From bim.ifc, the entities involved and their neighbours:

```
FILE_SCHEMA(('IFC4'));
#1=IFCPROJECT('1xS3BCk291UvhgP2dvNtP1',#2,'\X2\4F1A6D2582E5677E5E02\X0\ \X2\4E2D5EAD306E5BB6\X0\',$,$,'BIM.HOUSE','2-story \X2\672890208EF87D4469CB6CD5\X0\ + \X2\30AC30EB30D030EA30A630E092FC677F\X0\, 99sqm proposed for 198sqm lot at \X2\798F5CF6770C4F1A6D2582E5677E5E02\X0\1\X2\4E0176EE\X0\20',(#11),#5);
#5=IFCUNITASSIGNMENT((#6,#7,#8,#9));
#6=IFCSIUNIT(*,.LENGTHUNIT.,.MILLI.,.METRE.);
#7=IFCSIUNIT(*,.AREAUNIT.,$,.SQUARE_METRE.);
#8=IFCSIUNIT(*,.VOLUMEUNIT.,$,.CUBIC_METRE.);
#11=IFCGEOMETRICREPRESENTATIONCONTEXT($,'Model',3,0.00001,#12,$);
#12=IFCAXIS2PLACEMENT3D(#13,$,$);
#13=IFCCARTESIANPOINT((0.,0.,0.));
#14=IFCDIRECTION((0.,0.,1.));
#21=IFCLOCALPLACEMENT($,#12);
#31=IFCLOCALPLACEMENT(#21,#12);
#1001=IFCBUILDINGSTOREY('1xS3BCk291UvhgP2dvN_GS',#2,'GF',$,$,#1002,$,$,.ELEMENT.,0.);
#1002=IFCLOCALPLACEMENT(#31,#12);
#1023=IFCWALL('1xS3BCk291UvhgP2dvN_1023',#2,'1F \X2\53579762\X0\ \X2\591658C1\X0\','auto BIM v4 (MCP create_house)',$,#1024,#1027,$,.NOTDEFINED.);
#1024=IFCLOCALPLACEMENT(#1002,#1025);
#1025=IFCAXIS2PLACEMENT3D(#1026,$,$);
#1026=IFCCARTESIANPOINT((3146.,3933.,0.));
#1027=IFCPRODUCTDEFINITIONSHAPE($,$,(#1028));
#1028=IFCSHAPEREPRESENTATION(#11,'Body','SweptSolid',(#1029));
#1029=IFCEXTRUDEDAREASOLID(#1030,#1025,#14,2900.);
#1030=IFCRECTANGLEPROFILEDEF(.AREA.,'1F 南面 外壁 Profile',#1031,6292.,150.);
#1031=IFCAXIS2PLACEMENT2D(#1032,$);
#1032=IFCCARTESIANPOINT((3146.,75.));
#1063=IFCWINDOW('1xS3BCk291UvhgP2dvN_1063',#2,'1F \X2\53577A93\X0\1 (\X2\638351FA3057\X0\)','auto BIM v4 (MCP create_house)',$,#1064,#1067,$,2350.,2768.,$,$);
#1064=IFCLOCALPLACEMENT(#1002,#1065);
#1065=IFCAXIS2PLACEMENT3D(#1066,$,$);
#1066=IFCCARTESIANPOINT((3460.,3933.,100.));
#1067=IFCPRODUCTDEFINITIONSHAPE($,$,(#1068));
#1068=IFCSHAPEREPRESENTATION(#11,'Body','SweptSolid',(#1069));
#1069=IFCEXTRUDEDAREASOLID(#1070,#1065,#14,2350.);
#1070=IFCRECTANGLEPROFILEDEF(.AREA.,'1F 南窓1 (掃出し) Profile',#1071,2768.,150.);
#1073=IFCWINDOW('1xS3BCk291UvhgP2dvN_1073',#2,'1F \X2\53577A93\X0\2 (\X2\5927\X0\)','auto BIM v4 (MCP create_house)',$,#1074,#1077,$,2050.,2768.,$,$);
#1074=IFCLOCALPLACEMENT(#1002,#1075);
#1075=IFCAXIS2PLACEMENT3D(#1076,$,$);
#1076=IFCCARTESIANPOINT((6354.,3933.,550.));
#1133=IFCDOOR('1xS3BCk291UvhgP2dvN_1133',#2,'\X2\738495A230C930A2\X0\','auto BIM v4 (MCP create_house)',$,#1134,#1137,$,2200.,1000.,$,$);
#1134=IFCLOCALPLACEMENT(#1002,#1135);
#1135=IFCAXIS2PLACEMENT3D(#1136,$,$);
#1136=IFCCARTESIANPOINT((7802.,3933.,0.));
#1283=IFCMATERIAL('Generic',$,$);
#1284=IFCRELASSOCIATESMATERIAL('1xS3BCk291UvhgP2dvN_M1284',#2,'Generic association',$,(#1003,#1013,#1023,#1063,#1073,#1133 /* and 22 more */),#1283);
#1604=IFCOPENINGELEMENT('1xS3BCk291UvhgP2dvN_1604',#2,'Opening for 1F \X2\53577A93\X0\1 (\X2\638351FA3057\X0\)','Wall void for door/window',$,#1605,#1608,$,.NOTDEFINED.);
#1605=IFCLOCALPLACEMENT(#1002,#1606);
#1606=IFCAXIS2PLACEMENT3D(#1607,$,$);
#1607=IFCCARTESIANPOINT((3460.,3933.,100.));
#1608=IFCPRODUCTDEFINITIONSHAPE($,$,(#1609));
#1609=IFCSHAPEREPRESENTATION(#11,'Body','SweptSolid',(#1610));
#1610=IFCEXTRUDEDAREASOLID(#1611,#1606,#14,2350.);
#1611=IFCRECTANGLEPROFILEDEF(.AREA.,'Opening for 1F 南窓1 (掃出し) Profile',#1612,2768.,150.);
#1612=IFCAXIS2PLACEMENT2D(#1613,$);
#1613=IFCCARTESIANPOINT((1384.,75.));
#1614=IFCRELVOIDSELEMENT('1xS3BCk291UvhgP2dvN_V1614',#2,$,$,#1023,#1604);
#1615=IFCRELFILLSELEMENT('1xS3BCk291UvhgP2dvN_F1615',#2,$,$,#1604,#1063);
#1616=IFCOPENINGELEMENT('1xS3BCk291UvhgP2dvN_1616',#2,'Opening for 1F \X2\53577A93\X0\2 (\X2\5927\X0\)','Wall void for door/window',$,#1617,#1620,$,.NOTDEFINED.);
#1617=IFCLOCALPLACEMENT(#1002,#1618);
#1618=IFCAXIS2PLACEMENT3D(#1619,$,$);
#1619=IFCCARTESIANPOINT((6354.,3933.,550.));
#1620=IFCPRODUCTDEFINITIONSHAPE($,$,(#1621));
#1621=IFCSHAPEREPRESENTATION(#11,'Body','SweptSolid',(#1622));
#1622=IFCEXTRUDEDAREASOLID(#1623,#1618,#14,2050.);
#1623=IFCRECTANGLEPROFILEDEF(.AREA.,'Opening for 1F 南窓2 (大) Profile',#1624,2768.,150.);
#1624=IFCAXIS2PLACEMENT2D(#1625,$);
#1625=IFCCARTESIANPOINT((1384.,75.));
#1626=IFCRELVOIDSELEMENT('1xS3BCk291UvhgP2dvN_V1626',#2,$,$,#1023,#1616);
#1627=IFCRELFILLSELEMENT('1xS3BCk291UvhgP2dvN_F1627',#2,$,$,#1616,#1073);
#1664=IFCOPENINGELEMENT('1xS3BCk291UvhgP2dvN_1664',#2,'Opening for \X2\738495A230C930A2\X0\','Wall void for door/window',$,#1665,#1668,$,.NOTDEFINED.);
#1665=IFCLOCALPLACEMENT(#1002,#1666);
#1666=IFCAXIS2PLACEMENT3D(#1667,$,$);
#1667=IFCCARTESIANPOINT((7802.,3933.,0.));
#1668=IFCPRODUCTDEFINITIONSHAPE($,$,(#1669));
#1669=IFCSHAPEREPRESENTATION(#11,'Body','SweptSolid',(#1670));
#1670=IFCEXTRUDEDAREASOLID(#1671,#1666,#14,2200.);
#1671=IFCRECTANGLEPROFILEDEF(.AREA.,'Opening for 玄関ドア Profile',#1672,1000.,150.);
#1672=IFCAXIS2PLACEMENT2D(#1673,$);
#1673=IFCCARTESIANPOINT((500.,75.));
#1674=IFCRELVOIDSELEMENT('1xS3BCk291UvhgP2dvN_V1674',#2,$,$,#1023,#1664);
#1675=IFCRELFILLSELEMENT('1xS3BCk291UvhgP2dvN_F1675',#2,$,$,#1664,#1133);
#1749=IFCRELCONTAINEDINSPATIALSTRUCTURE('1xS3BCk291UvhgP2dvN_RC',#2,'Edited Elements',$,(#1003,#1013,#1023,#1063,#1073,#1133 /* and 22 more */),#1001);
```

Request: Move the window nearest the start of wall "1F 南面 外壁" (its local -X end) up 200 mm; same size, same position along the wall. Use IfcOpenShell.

```python
import numpy as np
import ifcopenshell
import ifcopenshell.api.geometry
import ifcopenshell.util.placement
import ifcopenshell.util.unit

model = ifcopenshell.open("bim.ifc")
unit_scale = ifcopenshell.util.unit.calculate_unit_scale(model)

window = model.by_id(1063)
opening = window.FillsVoids[0].RelatingOpeningElement
dz = 200.0

shift = np.array([0.0, 0.0, dz])
# The window is not placed relative to its opening, so move both.
for product in (opening, window):
    matrix = ifcopenshell.util.placement.get_local_placement(product.ObjectPlacement)
    matrix[:3, 3] += shift
    ifcopenshell.api.geometry.edit_object_placement(model, product=product, matrix=matrix, is_si=False)

print(f"moved by {dz * unit_scale:+.3f} m")

model.write("bim-out.ifc")
```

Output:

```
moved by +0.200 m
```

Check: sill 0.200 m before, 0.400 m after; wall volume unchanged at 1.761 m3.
